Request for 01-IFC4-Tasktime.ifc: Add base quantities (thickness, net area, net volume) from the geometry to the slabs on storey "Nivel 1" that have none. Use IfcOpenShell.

First a look at what the model holds.

```python
import ifcopenshell
import ifcopenshell.util.element
import ifcopenshell.util.unit

model = ifcopenshell.open("01-IFC4-Tasktime.ifc")
print(model.schema)
for unit_type in ("LENGTHUNIT", "AREAUNIT", "VOLUMEUNIT"):
    print(unit_type, ifcopenshell.util.unit.calculate_unit_scale(model, unit_type))
storey = next(s for s in model.by_type("IfcBuildingStorey") if s.Name == "Nivel 1")
slabs = [e for e in ifcopenshell.util.element.get_decomposition(storey) if e.is_a("IfcSlab")]
for e in sorted(slabs, key=lambda e: e.id()):
    print(e.id(), e.is_a(), e.Name, list(ifcopenshell.util.element.get_psets(e, qtos_only=True)), sep=" | ")
```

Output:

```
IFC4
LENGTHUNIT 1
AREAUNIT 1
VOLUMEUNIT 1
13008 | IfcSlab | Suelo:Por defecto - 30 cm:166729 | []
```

```python
import ifcopenshell
import ifcopenshell.api.pset
import ifcopenshell.geom
import ifcopenshell.util.element
import ifcopenshell.util.shape
import ifcopenshell.util.unit

model = ifcopenshell.open("01-IFC4-Tasktime.ifc")
unit_scale = ifcopenshell.util.unit.calculate_unit_scale(model)
area_scale = ifcopenshell.util.unit.calculate_unit_scale(model, "AREAUNIT")
volume_scale = ifcopenshell.util.unit.calculate_unit_scale(model, "VOLUMEUNIT")
settings = ifcopenshell.geom.settings()

storey = next(s for s in model.by_type("IfcBuildingStorey") if s.Name == "Nivel 1")
slabs = [e for e in ifcopenshell.util.element.get_decomposition(storey) if e.is_a("IfcSlab")]

for e in sorted(slabs, key=lambda e: e.id()):
    if ifcopenshell.util.element.get_psets(e, qtos_only=True, should_inherit=False):
        continue
    # Geometry comes back in metres, in the element's own axes.
    shape = ifcopenshell.geom.create_shape(settings, e)
    values = {
        "Width": ifcopenshell.util.shape.get_z(shape.geometry) / unit_scale,
        "NetArea": ifcopenshell.util.shape.get_footprint_area(shape.geometry) / area_scale,
        "NetVolume": ifcopenshell.util.shape.get_volume(shape.geometry) / volume_scale,
    }
    qto = ifcopenshell.api.pset.add_qto(model, product=e, name="Qto_SlabBaseQuantities")
    ifcopenshell.api.pset.edit_qto(model, qto=qto, properties=values)
    print(e.id(), {k: round(v, 3) for k, v in values.items()})

model.write("01-IFC4-Tasktime_v2.ifc")
```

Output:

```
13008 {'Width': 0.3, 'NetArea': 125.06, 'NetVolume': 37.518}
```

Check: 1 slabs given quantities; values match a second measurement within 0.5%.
